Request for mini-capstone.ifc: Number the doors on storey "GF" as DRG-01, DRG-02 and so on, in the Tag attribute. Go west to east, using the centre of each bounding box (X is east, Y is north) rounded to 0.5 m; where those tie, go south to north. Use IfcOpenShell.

First a look at what the model holds.

```python
import ifcopenshell
import ifcopenshell.util.element
import ifcopenshell.util.placement

model = ifcopenshell.open("mini-capstone.ifc")
print(model.schema)
storey = next(s for s in model.by_type("IfcBuildingStorey") if s.Name == "GF")
doors = [e for e in ifcopenshell.util.element.get_decomposition(storey) if e.is_a("IfcDoor")]
for e in sorted(doors, key=lambda e: e.id()):
    origin = ifcopenshell.util.placement.get_local_placement(e.ObjectPlacement)[:3, 3]
    print(e.id(), e.Tag, e.Name, origin.round(2) + 0.0, sep=" | ")
```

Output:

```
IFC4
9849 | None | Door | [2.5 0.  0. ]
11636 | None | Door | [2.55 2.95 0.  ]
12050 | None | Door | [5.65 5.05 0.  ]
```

```python
import ifcopenshell
import ifcopenshell.geom
import ifcopenshell.util.element
import ifcopenshell.util.shape

model = ifcopenshell.open("mini-capstone.ifc")
settings = ifcopenshell.geom.settings()
settings.set("use-world-coords", True)


def centre(element):
    shape = ifcopenshell.geom.create_shape(settings, element)
    return ifcopenshell.util.shape.get_bbox_centroid(shape.geometry)


storey = next(s for s in model.by_type("IfcBuildingStorey") if s.Name == "GF")
doors = [e for e in ifcopenshell.util.element.get_decomposition(storey) if e.is_a("IfcDoor")]

# Insertion points can sit at a corner or the storey origin, so sort by the geometry (in metres).
centres = {e: centre(e) for e in doors}
doors.sort(key=lambda e: (round(centres[e][0] / 0.5), centres[e][1]))

for i, e in enumerate(doors, start=1):
    number = f"DRG-{i:02d}"
    e.Tag = number
    print(e.id(), number)

model.write("mini-capstone-out.ifc")
```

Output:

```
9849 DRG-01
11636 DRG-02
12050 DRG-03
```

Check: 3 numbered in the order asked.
